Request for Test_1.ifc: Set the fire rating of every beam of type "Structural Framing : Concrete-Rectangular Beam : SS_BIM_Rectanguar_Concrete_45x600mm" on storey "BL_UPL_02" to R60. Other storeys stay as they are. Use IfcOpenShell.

First a look at what the model holds.

```python
import ifcopenshell
import ifcopenshell.util.element

model = ifcopenshell.open("Test_1.ifc")
print(model.schema)
storey = next(s for s in model.by_type("IfcBuildingStorey") if s.Name == "BL_UPL_02")
beams = [e for e in ifcopenshell.util.element.get_decomposition(storey) if e.is_a("IfcBeam")]
seen = {}
for e in beams:
    element_type = ifcopenshell.util.element.get_type(e)
    key = (element_type.Name if element_type != e and element_type else None, ifcopenshell.util.element.get_pset(e, "Pset_BeamCommon", "FireRating"))
    seen[key] = seen.get(key, 0) + 1
for (name, value), count in sorted(seen.items(), key=str):
    print(count, "x", name, "|", value)
```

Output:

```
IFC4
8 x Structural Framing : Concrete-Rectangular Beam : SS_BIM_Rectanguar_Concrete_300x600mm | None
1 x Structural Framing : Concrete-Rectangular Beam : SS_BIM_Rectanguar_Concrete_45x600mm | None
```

```python
import ifcopenshell
import ifcopenshell.api.pset
import ifcopenshell.util.element

model = ifcopenshell.open("Test_1.ifc")

storey = next(s for s in model.by_type("IfcBuildingStorey") if s.Name == "BL_UPL_02")
beams = [e for e in ifcopenshell.util.element.get_decomposition(storey) if e.is_a("IfcBeam")]

count = 0
for e in beams:
    element_type = ifcopenshell.util.element.get_type(e)
    if element_type in (None, e) or element_type.Name != "Structural Framing : Concrete-Rectangular Beam : SS_BIM_Rectanguar_Concrete_45x600mm":
        continue
    # add_pset returns the element's existing set when there is one.
    pset = ifcopenshell.api.pset.add_pset(model, product=e, name="Pset_BeamCommon")
    ifcopenshell.api.pset.edit_pset(model, pset=pset, properties={"FireRating": "R60"})
    count += 1

print(count, "beams updated")

model.write("Test_1-out.ifc")
```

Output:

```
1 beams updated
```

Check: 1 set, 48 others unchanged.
